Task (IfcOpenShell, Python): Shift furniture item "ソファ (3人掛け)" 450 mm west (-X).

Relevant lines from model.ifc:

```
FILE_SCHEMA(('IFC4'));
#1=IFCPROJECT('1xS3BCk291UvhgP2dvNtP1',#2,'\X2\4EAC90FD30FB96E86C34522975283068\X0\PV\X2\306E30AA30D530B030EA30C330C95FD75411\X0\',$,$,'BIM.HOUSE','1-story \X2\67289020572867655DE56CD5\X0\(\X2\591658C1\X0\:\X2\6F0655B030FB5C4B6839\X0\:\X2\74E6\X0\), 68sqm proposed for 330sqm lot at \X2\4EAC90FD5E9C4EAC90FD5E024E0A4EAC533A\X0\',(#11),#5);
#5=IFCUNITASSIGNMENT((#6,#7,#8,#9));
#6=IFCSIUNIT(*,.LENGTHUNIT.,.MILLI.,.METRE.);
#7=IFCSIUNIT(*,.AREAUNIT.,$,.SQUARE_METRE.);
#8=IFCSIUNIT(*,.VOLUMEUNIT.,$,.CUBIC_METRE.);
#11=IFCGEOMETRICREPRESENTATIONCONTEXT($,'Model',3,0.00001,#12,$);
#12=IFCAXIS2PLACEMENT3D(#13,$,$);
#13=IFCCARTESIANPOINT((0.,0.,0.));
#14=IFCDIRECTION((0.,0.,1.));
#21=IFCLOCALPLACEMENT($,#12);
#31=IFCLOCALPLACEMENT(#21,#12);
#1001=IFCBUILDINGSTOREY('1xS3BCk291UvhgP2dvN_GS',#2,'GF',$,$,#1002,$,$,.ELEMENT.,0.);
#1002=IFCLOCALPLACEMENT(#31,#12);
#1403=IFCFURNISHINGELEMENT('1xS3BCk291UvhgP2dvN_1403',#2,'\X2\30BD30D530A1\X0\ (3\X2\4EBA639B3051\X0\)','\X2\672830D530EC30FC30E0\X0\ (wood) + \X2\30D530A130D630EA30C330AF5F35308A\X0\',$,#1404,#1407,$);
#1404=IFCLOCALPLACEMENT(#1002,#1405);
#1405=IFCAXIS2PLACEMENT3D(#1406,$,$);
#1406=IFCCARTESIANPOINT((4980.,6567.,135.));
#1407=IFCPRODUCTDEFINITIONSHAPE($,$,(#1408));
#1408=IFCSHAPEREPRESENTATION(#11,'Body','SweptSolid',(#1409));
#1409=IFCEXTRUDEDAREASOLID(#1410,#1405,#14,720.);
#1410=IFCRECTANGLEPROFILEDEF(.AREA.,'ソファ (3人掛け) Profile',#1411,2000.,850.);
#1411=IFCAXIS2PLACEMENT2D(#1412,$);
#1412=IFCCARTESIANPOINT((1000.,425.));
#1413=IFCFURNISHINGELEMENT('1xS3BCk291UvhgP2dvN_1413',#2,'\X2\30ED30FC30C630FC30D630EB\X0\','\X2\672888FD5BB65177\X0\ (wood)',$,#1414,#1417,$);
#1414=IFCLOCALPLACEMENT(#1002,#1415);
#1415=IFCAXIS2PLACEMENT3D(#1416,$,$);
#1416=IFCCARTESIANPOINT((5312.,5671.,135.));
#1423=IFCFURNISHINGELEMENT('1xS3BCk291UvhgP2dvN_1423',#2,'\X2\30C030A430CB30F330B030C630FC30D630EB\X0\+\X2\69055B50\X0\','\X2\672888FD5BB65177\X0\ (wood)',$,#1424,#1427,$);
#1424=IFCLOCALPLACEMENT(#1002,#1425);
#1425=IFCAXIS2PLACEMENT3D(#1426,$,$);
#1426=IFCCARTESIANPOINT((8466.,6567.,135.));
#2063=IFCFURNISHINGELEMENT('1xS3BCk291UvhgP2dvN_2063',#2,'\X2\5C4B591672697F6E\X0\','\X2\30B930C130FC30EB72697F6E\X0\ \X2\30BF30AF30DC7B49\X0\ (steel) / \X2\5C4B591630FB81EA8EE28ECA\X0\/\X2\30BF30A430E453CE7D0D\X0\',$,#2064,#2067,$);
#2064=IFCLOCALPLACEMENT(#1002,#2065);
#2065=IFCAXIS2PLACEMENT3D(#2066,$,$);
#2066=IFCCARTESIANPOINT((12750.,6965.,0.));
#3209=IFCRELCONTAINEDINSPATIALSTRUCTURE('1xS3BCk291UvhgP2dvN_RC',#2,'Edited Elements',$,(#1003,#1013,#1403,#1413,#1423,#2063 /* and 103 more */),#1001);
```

```python
import ifcopenshell
import ifcopenshell.api.geometry
import ifcopenshell.util.placement
import ifcopenshell.util.unit

model = ifcopenshell.open("model.ifc")
unit_scale = ifcopenshell.util.unit.calculate_unit_scale(model)

item = model.by_guid("1xS3BCk291UvhgP2dvN_1403")
matrix = ifcopenshell.util.placement.get_local_placement(item.ObjectPlacement)
matrix[0, 3] -= 0.45 / unit_scale
ifcopenshell.api.geometry.edit_object_placement(model, product=item, matrix=matrix, is_si=False)

print(ifcopenshell.util.placement.get_local_placement(item.ObjectPlacement).round(3) + 0.0)

model.write("model-out.ifc")
```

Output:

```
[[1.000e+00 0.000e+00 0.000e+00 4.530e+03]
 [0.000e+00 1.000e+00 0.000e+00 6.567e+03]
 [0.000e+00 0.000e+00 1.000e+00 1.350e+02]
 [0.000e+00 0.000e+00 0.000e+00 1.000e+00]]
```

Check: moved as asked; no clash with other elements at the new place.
